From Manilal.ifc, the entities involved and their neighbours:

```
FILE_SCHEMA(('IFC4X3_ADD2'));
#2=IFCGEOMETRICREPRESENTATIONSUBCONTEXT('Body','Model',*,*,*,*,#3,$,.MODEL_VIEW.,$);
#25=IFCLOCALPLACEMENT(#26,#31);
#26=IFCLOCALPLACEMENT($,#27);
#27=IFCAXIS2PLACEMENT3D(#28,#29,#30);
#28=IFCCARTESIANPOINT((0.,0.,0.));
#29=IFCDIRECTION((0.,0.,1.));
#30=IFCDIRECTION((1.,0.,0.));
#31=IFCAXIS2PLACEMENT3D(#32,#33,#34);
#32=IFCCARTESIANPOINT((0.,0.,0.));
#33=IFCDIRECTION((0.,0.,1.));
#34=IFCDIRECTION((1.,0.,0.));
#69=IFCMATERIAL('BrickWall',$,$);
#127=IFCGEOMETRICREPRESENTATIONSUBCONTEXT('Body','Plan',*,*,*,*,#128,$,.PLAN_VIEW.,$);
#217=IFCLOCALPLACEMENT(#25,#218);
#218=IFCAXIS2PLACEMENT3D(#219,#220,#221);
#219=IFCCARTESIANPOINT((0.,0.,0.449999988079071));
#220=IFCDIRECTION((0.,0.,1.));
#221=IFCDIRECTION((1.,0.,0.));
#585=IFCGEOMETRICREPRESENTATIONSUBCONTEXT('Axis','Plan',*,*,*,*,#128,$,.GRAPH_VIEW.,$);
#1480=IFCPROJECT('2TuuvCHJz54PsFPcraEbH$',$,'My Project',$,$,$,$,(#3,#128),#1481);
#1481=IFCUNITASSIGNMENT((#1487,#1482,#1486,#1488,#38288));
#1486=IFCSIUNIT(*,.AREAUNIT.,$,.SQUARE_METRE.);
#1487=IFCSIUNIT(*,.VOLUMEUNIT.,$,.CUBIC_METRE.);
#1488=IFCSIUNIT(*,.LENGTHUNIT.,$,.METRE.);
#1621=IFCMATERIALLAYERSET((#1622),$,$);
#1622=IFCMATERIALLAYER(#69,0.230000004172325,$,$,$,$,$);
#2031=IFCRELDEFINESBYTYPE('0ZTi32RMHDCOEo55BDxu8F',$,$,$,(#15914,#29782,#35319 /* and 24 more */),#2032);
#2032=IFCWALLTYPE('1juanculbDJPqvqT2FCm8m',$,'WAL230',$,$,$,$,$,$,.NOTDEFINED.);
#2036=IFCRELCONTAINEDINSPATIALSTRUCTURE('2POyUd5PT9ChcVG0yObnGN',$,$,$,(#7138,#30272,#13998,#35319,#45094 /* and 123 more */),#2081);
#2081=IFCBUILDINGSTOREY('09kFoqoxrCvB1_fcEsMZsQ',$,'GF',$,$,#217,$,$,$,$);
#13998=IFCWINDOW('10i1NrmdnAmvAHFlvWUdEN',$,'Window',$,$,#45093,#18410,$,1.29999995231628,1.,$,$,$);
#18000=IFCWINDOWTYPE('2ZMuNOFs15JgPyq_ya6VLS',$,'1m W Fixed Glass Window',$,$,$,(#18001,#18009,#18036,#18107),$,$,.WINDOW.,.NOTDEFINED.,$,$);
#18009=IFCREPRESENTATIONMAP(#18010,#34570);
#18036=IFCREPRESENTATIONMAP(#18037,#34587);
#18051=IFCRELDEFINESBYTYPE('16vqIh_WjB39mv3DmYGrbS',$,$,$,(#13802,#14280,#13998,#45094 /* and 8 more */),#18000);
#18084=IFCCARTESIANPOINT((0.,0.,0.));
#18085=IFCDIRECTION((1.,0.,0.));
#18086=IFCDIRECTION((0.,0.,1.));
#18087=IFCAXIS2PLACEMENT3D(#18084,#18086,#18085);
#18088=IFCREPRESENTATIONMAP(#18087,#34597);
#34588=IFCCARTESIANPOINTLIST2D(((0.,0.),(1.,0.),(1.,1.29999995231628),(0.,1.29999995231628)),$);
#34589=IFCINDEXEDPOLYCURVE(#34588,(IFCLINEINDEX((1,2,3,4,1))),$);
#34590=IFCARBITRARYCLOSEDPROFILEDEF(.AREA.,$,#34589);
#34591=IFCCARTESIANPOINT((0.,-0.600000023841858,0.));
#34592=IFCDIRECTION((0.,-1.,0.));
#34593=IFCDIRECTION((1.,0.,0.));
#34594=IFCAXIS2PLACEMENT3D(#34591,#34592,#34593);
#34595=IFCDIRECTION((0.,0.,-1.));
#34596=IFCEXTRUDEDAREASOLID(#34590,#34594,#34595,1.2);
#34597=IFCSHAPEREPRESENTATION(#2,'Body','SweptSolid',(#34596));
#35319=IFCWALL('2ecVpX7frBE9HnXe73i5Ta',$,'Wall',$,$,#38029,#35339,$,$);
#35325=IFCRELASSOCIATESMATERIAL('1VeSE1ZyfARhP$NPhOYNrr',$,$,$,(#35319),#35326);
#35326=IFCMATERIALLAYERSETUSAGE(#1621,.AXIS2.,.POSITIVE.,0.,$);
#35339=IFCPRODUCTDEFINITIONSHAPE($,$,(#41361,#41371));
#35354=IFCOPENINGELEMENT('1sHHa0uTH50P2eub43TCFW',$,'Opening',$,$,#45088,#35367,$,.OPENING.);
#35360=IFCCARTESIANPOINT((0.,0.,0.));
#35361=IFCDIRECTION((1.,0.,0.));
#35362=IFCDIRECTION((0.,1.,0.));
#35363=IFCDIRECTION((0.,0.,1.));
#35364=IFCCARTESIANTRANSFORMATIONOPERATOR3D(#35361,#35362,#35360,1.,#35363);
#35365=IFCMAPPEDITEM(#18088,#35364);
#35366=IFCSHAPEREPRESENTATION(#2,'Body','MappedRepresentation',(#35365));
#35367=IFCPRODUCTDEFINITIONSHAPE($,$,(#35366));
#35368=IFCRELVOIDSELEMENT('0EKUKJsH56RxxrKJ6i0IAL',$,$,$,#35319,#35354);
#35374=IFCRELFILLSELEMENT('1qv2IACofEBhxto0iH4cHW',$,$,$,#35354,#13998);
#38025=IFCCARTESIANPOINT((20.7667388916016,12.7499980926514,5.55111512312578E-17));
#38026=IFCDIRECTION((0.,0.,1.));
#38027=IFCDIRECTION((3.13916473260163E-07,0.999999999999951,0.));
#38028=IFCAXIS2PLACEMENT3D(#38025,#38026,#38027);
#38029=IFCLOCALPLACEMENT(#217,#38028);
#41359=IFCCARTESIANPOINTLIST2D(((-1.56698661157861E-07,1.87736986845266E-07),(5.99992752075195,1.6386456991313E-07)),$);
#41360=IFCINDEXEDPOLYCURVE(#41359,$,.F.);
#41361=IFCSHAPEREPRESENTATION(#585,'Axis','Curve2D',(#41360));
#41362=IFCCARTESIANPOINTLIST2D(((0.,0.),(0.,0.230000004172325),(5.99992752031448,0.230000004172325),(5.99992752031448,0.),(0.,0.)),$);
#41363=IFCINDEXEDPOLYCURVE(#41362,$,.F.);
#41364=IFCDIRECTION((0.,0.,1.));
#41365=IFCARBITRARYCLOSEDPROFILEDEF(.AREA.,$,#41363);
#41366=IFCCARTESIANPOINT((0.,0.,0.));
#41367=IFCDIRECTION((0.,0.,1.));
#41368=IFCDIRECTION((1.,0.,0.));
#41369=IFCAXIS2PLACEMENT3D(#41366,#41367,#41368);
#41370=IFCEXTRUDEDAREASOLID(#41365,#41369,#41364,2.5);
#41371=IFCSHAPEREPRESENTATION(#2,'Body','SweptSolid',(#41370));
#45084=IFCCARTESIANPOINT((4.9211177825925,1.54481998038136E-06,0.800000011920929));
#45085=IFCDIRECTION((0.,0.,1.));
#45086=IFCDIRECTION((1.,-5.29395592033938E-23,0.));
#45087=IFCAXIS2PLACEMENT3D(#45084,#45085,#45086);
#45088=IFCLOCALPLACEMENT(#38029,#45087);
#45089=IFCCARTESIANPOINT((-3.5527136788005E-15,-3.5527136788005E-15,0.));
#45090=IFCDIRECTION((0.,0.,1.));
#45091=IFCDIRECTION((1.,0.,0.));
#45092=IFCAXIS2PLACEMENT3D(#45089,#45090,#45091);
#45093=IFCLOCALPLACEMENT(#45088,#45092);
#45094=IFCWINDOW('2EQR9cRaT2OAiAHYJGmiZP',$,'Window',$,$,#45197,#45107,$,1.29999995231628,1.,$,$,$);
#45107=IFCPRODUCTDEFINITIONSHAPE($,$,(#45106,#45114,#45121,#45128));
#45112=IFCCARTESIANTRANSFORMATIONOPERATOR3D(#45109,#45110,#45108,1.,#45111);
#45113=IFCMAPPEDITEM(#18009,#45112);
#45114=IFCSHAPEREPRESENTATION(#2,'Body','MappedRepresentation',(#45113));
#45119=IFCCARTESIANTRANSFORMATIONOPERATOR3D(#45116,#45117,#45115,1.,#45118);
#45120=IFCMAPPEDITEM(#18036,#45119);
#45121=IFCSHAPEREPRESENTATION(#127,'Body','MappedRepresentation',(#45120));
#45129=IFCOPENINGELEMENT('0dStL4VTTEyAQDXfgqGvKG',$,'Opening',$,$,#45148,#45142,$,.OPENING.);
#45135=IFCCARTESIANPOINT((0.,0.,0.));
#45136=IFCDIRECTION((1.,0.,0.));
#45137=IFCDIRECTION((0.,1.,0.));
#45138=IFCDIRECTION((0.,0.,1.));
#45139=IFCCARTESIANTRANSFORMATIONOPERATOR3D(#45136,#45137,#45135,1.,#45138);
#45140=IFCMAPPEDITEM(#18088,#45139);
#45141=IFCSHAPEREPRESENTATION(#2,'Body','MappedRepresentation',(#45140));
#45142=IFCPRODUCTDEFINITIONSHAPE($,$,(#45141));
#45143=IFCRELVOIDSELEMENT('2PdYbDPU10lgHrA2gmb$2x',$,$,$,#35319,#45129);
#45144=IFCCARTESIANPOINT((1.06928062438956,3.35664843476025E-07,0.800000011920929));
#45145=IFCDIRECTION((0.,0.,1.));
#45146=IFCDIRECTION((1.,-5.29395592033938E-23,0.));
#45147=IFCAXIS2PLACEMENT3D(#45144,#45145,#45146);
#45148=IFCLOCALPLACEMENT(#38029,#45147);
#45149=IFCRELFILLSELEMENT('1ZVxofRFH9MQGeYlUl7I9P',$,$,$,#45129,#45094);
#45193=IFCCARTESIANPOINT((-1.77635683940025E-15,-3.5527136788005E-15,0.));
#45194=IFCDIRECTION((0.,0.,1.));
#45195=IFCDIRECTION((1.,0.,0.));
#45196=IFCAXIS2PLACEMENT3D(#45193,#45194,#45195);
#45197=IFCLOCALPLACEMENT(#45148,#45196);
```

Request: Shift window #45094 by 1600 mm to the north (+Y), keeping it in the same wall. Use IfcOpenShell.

```python
import ifcopenshell
import ifcopenshell.api.geometry
import ifcopenshell.util.placement
import ifcopenshell.util.unit

model = ifcopenshell.open("Manilal.ifc")
unit_scale = ifcopenshell.util.unit.calculate_unit_scale(model)

window = model.by_guid("2EQR9cRaT2OAiAHYJGmiZP")
opening = window.FillsVoids[0].RelatingOpeningElement
wall = opening.VoidsElements[0].RelatingBuildingElement

wall_matrix = ifcopenshell.util.placement.get_local_placement(wall.ObjectPlacement)
shift = wall_matrix[:3, 0] * 1.6 / unit_scale
before = ifcopenshell.util.placement.get_local_placement(window.ObjectPlacement)[:3, 3].copy()

# The window is placed relative to its opening, so it follows when the opening moves.
matrix = ifcopenshell.util.placement.get_local_placement(opening.ObjectPlacement)
matrix[:3, 3] += shift
ifcopenshell.api.geometry.edit_object_placement(
    model, product=opening, matrix=matrix, is_si=False, should_transform_children=True
)

after = ifcopenshell.util.placement.get_local_placement(window.ObjectPlacement)[:3, 3]
print("window moved by", (after - before).round(3) + 0.0)

model.write("Manilal-out.ifc")
```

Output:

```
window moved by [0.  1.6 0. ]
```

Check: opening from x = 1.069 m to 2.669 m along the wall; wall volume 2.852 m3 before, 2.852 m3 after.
